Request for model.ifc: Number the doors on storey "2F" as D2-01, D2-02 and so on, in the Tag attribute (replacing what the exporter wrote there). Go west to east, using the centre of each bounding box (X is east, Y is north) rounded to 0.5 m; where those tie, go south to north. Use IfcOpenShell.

First a look at what the model holds.

```python
import ifcopenshell
import ifcopenshell.util.element
import ifcopenshell.util.placement

model = ifcopenshell.open("model.ifc")
print(model.schema)
storey = next(s for s in model.by_type("IfcBuildingStorey") if s.Name == "2F")
doors = [e for e in ifcopenshell.util.element.get_decomposition(storey) if e.is_a("IfcDoor")]
for e in sorted(doors, key=lambda e: e.id()):
    origin = ifcopenshell.util.placement.get_local_placement(e.ObjectPlacement)[:3, 3]
    print(e.id(), e.Tag, e.Name, origin.round(2) + 0.0, sep=" | ")
```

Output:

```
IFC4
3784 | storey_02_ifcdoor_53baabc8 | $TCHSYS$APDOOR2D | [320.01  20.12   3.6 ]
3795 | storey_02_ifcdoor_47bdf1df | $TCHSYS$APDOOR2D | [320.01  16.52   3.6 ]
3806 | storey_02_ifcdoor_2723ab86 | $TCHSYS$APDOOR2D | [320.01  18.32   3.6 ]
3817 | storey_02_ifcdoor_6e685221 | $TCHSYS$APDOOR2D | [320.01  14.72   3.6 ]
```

```python
import ifcopenshell
import ifcopenshell.geom
import ifcopenshell.util.element
import ifcopenshell.util.shape

model = ifcopenshell.open("model.ifc")
settings = ifcopenshell.geom.settings()
settings.set("use-world-coords", True)


def centre(element):
    shape = ifcopenshell.geom.create_shape(settings, element)
    return ifcopenshell.util.shape.get_bbox_centroid(shape.geometry)


storey = next(s for s in model.by_type("IfcBuildingStorey") if s.Name == "2F")
doors = [e for e in ifcopenshell.util.element.get_decomposition(storey) if e.is_a("IfcDoor")]

# Insertion points can sit at a corner or the storey origin, so sort by the geometry (in metres).
centres = {e: centre(e) for e in doors}
doors.sort(key=lambda e: (round(centres[e][0] / 0.5), centres[e][1]))

for i, e in enumerate(doors, start=1):
    number = f"D2-{i:02d}"
    e.Tag = number
    print(e.id(), number)

model.write("model-out.ifc")
```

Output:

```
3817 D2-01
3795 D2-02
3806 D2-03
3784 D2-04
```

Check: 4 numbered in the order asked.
